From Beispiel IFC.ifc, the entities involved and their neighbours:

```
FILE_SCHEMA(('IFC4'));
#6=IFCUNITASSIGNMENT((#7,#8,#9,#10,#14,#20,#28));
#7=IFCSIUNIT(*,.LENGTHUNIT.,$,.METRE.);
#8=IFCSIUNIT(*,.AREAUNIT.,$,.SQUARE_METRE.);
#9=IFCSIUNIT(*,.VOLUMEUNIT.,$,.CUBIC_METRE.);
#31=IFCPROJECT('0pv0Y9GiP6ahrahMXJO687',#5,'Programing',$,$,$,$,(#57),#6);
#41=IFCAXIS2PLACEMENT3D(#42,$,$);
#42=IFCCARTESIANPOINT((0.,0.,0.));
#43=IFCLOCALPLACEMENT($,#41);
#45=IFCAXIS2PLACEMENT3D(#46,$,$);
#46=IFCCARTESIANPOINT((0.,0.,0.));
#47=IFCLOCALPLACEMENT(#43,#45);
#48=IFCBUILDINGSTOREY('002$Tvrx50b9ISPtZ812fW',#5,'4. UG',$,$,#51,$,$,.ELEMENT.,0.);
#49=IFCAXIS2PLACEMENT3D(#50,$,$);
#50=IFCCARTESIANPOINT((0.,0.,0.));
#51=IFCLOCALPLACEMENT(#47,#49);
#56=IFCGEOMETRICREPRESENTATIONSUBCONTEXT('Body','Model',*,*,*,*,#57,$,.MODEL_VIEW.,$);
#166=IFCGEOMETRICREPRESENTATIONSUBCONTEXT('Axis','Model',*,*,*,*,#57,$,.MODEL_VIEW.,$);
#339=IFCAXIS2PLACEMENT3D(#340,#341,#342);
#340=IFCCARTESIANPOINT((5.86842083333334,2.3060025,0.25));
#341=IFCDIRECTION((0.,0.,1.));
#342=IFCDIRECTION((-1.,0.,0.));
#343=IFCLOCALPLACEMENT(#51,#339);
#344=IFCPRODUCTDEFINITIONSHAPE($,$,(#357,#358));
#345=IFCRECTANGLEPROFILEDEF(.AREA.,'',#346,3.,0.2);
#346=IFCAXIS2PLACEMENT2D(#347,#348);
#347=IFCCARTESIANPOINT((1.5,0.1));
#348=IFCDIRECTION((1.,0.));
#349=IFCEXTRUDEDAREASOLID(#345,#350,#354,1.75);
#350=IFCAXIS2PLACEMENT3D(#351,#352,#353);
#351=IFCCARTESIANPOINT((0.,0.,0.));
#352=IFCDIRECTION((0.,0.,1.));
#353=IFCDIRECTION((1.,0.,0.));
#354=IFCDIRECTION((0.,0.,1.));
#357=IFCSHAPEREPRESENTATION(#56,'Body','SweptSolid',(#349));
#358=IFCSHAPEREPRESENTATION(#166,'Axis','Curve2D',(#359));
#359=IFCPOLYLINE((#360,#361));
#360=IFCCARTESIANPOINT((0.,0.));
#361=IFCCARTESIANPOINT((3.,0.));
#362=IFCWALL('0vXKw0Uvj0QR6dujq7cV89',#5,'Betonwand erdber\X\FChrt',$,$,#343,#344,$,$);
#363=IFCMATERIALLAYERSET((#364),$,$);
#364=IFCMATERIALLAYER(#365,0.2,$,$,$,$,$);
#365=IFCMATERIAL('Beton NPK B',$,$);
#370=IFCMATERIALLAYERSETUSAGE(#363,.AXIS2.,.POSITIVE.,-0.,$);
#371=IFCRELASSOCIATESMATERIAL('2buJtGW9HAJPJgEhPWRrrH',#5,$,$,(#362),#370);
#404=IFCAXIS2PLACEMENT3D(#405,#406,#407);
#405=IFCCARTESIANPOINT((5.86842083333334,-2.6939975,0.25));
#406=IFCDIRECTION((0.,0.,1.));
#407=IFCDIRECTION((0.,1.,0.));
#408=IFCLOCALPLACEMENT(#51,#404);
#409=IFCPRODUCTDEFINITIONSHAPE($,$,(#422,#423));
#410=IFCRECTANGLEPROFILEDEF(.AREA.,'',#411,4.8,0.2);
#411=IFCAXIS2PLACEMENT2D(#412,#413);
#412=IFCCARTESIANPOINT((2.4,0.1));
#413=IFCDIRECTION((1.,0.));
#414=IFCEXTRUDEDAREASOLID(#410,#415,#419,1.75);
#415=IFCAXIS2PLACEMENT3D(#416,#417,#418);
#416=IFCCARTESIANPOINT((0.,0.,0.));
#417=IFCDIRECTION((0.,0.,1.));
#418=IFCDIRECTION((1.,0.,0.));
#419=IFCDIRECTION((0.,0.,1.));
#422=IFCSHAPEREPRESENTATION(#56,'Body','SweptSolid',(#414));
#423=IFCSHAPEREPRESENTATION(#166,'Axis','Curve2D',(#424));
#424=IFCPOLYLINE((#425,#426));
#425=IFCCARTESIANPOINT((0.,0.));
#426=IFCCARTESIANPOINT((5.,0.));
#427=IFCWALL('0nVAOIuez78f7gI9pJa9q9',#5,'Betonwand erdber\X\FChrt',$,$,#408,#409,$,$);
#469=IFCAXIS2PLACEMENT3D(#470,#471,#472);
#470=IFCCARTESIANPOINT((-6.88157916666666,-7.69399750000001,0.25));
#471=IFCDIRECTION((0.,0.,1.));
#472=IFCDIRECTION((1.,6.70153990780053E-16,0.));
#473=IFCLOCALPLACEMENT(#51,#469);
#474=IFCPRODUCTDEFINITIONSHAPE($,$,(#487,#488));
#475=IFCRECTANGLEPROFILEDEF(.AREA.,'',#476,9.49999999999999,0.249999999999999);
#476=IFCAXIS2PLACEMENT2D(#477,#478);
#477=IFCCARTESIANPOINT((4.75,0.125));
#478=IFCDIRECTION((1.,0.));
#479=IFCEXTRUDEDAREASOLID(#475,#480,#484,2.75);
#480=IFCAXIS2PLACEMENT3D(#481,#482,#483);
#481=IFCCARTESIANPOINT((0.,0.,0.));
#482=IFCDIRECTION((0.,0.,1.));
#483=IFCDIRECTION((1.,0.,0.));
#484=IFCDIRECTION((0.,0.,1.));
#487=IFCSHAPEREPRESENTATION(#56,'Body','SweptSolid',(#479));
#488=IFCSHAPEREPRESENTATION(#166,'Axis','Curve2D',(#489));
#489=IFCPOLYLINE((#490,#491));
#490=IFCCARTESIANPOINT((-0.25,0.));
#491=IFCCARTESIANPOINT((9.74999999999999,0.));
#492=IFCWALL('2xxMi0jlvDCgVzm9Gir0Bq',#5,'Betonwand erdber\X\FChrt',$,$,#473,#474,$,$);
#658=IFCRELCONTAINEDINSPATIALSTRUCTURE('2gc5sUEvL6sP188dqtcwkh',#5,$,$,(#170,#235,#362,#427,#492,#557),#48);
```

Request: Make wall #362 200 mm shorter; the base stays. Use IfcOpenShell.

```python
import ifcopenshell
import ifcopenshell.geom
import ifcopenshell.util.representation
import ifcopenshell.util.shape
import ifcopenshell.util.unit

model = ifcopenshell.open("Beispiel IFC.ifc")
unit_scale = ifcopenshell.util.unit.calculate_unit_scale(model)
settings = ifcopenshell.geom.settings()


def volume(element):
    """Net volume in cubic metres, openings subtracted."""
    shape = ifcopenshell.geom.create_shape(settings, element)
    return ifcopenshell.util.shape.get_volume(shape.geometry)


wall = model.by_id(362)
before = volume(wall)

body = ifcopenshell.util.representation.get_representation(wall, "Model", "Body")
solid = body.Items[0]
old_height = solid.Depth
solid.Depth -= 0.2 / unit_scale
after = volume(wall)

print(f"height {old_height:g} -> {solid.Depth:g}, volume {before:.3f} -> {after:.3f} m3")

model.write("Beispiel IFC-out.ifc")
```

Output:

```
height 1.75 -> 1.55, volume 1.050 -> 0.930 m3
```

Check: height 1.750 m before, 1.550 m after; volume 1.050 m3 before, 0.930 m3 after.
